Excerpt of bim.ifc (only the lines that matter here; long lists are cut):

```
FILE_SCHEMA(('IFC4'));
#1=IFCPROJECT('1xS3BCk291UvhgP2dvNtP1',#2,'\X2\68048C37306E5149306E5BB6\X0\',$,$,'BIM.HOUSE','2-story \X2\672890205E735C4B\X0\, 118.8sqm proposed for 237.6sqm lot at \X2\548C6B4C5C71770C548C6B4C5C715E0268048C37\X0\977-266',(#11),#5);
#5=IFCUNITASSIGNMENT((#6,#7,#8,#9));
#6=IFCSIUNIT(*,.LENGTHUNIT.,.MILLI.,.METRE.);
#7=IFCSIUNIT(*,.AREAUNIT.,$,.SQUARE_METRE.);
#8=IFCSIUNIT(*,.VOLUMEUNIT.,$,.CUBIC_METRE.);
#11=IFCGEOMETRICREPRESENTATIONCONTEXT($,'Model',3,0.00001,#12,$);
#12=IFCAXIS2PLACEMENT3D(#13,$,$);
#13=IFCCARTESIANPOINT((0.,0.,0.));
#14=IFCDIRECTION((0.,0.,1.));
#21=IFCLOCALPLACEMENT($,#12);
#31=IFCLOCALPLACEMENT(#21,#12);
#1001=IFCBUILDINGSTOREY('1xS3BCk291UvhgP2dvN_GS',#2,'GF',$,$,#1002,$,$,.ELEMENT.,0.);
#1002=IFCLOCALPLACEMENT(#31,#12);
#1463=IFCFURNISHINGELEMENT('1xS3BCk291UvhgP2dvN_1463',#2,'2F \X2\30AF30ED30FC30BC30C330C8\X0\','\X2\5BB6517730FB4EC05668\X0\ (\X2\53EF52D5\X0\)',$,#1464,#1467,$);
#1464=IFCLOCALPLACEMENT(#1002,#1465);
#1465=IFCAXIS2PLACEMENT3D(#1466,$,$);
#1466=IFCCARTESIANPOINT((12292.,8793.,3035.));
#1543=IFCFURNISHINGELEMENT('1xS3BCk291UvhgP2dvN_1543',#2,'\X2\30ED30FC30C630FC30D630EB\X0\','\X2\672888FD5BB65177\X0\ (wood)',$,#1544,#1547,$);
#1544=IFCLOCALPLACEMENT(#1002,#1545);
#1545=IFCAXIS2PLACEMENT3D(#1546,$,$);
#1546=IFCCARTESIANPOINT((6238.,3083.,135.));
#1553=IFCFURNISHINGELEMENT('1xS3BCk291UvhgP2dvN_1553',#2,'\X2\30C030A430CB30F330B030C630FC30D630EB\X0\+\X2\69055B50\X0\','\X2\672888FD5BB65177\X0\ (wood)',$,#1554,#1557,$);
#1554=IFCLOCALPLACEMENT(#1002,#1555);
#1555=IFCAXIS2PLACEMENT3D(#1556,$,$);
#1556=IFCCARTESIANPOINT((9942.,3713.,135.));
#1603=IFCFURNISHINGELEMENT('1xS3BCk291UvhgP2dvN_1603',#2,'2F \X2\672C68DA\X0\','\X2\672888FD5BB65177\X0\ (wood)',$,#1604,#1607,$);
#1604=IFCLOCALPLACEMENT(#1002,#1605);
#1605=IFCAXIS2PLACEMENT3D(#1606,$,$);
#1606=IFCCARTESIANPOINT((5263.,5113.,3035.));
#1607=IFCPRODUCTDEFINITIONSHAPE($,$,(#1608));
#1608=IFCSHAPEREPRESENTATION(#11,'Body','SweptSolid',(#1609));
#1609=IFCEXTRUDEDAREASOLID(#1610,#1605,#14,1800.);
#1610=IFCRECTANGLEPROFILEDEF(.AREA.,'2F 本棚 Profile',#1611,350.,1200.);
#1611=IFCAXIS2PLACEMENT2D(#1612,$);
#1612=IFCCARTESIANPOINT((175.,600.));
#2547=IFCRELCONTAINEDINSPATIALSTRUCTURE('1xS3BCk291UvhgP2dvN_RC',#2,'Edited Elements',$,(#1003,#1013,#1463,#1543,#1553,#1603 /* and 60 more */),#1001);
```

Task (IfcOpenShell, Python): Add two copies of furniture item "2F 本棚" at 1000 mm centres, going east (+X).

```python
import numpy as np
import ifcopenshell
import ifcopenshell.api.geometry
import ifcopenshell.api.root
import ifcopenshell.util.element
import ifcopenshell.util.placement

model = ifcopenshell.open("bim.ifc")


def reuse_history(source, copy):
    """copy_class also copies each property set's owner history, people and application; keep the originals."""
    for rel in copy.IsDefinedBy:
        if rel.is_a("IfcRelDefinesByProperties") and (history := rel.RelatingPropertyDefinition.OwnerHistory):
            rel.RelatingPropertyDefinition.OwnerHistory = source.OwnerHistory
            ifcopenshell.util.element.remove_deep2(model, history)


source = model.by_guid("1xS3BCk291UvhgP2dvN_1603")
base = ifcopenshell.util.placement.get_local_placement(source.ObjectPlacement)
step = np.array([1.0, 0.0, 0.0]) * 1000.0

for i in range(1, 3):
    copy = ifcopenshell.api.root.copy_class(model, product=source)
    copy.Representation = ifcopenshell.util.element.copy_deep(
        model, source.Representation, exclude=["IfcGeometricRepresentationContext", "IfcRepresentationMap"]
    )
    reuse_history(source, copy)
    matrix = base.copy()
    matrix[:3, 3] += i * step
    print("added at", matrix[:3, 3].round(3) + 0.0)
    ifcopenshell.api.geometry.edit_object_placement(model, product=copy, matrix=matrix, is_si=False)

model.write("bim_edited.ifc")
```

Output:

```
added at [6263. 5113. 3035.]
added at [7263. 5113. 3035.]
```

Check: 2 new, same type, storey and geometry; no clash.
